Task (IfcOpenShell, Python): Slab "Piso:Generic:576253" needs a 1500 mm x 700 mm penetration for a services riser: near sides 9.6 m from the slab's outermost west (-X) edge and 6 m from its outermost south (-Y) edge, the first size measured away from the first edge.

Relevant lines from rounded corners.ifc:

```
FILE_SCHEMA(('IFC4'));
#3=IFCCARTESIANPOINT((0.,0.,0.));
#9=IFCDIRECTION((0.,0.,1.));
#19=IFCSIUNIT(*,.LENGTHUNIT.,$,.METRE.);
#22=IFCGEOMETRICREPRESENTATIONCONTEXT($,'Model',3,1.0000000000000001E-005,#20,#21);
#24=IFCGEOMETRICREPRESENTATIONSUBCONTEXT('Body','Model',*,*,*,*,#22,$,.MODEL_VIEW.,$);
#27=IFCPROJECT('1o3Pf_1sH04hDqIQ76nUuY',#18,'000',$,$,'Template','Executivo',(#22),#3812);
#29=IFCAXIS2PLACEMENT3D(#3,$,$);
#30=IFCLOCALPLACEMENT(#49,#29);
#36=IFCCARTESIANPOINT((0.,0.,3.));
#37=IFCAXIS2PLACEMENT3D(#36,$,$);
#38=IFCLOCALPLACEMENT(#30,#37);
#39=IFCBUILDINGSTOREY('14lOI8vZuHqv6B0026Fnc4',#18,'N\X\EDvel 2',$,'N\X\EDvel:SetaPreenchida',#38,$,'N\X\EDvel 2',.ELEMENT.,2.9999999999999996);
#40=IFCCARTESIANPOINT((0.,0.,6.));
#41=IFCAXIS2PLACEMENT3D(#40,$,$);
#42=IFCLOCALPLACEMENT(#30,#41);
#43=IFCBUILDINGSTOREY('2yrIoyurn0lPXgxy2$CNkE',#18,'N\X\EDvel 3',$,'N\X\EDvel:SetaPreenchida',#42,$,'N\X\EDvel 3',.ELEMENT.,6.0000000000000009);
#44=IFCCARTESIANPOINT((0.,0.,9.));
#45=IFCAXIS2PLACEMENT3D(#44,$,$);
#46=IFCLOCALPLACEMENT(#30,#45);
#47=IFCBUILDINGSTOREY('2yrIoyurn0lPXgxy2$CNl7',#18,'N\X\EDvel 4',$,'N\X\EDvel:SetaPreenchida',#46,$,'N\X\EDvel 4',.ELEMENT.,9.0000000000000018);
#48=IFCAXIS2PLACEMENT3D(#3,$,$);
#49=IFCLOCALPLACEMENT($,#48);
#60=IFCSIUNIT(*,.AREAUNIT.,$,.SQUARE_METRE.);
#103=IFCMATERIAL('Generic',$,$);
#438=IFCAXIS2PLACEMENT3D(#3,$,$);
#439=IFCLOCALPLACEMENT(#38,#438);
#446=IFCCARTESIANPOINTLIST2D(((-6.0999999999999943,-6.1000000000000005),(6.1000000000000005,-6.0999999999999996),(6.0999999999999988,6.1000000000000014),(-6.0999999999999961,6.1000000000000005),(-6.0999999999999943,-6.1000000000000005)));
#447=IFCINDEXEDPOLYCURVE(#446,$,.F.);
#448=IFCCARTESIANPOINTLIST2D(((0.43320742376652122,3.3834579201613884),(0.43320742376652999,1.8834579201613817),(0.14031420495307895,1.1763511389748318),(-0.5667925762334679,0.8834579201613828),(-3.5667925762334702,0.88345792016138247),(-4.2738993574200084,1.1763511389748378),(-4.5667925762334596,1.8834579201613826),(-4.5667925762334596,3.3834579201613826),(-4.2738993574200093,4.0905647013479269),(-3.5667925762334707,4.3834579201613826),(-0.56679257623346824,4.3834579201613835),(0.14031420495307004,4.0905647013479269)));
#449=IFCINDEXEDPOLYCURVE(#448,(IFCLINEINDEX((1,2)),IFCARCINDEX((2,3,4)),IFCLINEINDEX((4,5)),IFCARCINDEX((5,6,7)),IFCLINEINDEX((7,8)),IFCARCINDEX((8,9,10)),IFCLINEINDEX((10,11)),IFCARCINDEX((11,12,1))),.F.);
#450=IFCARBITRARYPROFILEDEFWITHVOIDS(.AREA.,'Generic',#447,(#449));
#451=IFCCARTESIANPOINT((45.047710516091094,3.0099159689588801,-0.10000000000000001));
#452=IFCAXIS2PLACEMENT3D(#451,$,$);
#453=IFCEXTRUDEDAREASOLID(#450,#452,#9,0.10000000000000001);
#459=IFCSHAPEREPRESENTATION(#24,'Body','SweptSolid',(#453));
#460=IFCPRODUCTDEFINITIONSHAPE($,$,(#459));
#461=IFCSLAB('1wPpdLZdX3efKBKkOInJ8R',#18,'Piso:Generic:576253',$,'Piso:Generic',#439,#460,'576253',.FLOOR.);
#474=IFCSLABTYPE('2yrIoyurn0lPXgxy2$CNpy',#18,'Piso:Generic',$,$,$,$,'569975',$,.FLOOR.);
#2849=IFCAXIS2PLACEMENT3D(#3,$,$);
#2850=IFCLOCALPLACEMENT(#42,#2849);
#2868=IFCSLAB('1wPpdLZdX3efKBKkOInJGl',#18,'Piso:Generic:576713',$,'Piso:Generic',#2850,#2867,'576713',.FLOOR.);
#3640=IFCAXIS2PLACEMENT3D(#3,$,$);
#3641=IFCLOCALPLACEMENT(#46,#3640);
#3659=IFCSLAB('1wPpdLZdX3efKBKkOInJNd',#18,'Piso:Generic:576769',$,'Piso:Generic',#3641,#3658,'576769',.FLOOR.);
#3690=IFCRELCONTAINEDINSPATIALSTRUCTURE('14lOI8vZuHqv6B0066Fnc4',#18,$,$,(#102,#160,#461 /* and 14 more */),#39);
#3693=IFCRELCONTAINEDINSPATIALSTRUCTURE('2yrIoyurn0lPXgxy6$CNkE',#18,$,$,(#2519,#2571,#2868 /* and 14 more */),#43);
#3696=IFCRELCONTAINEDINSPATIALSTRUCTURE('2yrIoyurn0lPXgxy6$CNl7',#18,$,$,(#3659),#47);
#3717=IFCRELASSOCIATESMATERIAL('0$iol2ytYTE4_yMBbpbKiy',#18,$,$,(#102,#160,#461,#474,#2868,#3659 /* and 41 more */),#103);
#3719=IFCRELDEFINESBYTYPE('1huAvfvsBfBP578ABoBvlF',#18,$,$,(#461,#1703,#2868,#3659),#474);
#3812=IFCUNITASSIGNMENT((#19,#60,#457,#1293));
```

```python
import numpy as np
import ifcopenshell
import ifcopenshell.api.feature
import ifcopenshell.api.geometry
import ifcopenshell.api.root
import ifcopenshell.geom
import ifcopenshell.util.placement
import ifcopenshell.util.representation
import ifcopenshell.util.shape
import ifcopenshell.util.unit

model = ifcopenshell.open("rounded corners.ifc")
unit_scale = ifcopenshell.util.unit.calculate_unit_scale(model)
settings = ifcopenshell.geom.settings()


def volume(element):
    """Net volume in cubic metres, openings subtracted."""
    shape = ifcopenshell.geom.create_shape(settings, element)
    return ifcopenshell.util.shape.get_volume(shape.geometry)


slab = model.by_id(461)
before = volume(slab)

# Extent in the slab's own axes, in metres. The edges named are its -X and -Y sides.
slab_shape = ifcopenshell.geom.create_shape(settings, slab)
vertices = ifcopenshell.util.shape.get_vertices(slab_shape.geometry)
x_min, y_min, bottom = vertices.min(axis=0)
top = vertices[:, 2].max()

opening = ifcopenshell.api.root.create_entity(model, ifc_class="IfcOpeningElement", name="Services riser opening", predefined_type="OPENING")
context = ifcopenshell.util.representation.get_context(model, "Model", "Body", "MODEL_VIEW")
width, depth = 1.5, 0.7
outline = [(0.0, 0.0), (width, 0.0), (width, depth), (0.0, depth), (0.0, 0.0)]
# Overshoot both faces by 50 mm so the cut is clean.
shape = ifcopenshell.api.geometry.add_slab_representation(
    model, context=context, depth=top - bottom + 0.1, polyline=outline
)
ifcopenshell.api.geometry.assign_representation(model, product=opening, representation=shape)

matrix = ifcopenshell.util.placement.get_local_placement(slab.ObjectPlacement)
matrix[:, 3] = matrix @ np.append(np.array([x_min + 9.6, y_min + 6, bottom - 0.05]) / unit_scale, 1.0)
ifcopenshell.api.geometry.edit_object_placement(model, product=opening, matrix=matrix, is_si=False)
ifcopenshell.api.feature.add_feature(model, feature=opening, element=slab)

after = volume(slab)

print(f"slab volume {before:.3f} -> {after:.3f} m3")

model.write("rounded corners_rev.ifc")
```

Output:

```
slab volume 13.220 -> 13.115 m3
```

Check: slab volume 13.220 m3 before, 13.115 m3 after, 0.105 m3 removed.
